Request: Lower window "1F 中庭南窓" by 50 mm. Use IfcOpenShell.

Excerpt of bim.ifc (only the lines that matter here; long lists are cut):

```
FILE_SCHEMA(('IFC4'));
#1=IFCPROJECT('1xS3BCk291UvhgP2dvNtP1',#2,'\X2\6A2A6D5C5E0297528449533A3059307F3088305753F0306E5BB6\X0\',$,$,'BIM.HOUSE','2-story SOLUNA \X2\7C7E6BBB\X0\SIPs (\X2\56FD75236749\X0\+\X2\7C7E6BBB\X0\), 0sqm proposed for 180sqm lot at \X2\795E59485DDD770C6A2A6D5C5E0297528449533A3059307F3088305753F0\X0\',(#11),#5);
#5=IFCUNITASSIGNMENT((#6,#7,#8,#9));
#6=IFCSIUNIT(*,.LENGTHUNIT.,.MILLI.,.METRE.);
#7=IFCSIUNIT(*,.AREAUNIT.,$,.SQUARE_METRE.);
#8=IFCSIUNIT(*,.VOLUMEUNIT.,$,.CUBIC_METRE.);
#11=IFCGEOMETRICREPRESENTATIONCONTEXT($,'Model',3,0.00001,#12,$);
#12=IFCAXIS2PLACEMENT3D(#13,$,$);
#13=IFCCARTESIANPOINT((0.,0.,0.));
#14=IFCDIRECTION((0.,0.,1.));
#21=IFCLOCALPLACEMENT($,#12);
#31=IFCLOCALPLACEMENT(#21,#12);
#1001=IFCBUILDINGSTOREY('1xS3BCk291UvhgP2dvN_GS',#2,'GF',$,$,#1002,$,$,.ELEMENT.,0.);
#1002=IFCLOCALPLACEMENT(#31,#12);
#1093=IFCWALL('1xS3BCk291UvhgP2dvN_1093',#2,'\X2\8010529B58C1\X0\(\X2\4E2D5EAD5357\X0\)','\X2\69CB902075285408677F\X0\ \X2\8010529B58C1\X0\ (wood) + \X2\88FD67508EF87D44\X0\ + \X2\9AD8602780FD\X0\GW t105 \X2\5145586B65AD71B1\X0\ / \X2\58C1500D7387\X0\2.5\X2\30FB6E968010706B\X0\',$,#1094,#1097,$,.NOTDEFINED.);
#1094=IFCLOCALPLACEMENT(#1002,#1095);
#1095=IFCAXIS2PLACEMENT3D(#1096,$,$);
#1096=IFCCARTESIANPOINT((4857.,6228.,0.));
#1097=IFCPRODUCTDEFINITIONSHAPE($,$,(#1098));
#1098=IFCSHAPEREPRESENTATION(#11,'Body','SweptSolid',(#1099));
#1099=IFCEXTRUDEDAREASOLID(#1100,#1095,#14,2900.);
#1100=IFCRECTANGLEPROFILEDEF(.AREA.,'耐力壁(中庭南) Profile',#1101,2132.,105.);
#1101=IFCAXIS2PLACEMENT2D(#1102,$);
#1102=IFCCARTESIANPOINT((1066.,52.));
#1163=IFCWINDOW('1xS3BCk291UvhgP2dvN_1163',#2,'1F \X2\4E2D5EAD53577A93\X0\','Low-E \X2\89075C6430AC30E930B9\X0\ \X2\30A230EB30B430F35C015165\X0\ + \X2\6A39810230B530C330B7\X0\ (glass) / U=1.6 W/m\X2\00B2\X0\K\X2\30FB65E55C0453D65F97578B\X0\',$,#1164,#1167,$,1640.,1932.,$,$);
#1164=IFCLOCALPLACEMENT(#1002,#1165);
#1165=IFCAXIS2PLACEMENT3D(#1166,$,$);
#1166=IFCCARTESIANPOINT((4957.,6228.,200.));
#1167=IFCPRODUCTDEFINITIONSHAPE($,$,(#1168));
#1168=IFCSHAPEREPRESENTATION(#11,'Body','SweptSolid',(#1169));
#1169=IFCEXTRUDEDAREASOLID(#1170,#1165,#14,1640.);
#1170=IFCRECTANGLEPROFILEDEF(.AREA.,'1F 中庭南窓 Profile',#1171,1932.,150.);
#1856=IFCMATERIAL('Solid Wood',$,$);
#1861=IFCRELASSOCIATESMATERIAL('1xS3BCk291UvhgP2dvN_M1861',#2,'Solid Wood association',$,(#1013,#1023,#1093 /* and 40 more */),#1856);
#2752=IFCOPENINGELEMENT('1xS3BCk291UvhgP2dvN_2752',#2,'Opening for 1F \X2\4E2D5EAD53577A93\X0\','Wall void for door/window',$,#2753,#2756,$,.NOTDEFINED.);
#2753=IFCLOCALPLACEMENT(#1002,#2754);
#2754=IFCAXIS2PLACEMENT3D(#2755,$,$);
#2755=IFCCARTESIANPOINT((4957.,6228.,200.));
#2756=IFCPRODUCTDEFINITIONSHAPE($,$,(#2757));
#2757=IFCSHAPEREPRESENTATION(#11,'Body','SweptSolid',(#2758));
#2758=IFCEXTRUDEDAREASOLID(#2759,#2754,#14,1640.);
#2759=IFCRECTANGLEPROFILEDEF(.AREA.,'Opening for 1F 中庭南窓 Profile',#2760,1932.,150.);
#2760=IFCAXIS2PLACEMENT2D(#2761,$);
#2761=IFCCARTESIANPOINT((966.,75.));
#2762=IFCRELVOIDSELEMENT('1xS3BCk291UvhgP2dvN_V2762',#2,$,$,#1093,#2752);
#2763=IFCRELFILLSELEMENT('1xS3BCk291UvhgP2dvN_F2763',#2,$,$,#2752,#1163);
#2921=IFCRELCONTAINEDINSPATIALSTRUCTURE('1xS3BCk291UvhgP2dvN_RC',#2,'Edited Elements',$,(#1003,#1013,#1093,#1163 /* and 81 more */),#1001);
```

```python
import numpy as np
import ifcopenshell
import ifcopenshell.api.geometry
import ifcopenshell.util.placement
import ifcopenshell.util.unit

model = ifcopenshell.open("bim.ifc")
unit_scale = ifcopenshell.util.unit.calculate_unit_scale(model)

window = model.by_guid("1xS3BCk291UvhgP2dvN_1163")
opening = window.FillsVoids[0].RelatingOpeningElement
dz = -50.0

shift = np.array([0.0, 0.0, dz])
# The window is not placed relative to its opening, so move both.
for product in (opening, window):
    matrix = ifcopenshell.util.placement.get_local_placement(product.ObjectPlacement)
    matrix[:3, 3] += shift
    ifcopenshell.api.geometry.edit_object_placement(model, product=product, matrix=matrix, is_si=False)

print(f"moved by {dz * unit_scale:+.3f} m")

model.write("bim_v2.ifc")
```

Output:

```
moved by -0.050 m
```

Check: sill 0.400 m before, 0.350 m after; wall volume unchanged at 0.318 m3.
